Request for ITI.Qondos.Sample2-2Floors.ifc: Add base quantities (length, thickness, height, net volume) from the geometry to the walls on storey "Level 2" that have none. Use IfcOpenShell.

First a look at what the model holds.

```python
import ifcopenshell
import ifcopenshell.util.element
import ifcopenshell.util.unit

model = ifcopenshell.open("ITI.Qondos.Sample2-2Floors.ifc")
print(model.schema)
for unit_type in ("LENGTHUNIT", "AREAUNIT", "VOLUMEUNIT"):
    print(unit_type, ifcopenshell.util.unit.calculate_unit_scale(model, unit_type))
storey = next(s for s in model.by_type("IfcBuildingStorey") if s.Name == "Level 2")
walls = [e for e in ifcopenshell.util.element.get_decomposition(storey) if e.is_a("IfcWall")]
for e in sorted(walls, key=lambda e: e.id()):
    print(e.id(), e.is_a(), e.Name, list(ifcopenshell.util.element.get_psets(e, qtos_only=True)), sep=" | ")
```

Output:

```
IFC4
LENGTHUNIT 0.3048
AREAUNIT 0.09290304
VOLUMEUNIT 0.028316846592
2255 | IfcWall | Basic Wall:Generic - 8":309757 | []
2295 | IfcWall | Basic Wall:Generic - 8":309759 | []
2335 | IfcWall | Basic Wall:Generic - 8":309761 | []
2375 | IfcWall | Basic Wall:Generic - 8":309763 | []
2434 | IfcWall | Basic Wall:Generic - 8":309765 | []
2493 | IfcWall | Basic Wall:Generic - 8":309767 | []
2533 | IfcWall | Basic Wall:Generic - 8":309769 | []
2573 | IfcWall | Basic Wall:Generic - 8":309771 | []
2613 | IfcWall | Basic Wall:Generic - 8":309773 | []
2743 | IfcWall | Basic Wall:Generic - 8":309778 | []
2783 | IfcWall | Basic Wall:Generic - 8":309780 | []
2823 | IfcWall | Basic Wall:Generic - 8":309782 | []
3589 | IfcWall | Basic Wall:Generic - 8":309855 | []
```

```python
import ifcopenshell
import ifcopenshell.api.pset
import ifcopenshell.geom
import ifcopenshell.util.element
import ifcopenshell.util.shape
import ifcopenshell.util.unit

model = ifcopenshell.open("ITI.Qondos.Sample2-2Floors.ifc")
unit_scale = ifcopenshell.util.unit.calculate_unit_scale(model)
volume_scale = ifcopenshell.util.unit.calculate_unit_scale(model, "VOLUMEUNIT")
settings = ifcopenshell.geom.settings()

storey = next(s for s in model.by_type("IfcBuildingStorey") if s.Name == "Level 2")
walls = [e for e in ifcopenshell.util.element.get_decomposition(storey) if e.is_a("IfcWall")]

for e in sorted(walls, key=lambda e: e.id()):
    if ifcopenshell.util.element.get_psets(e, qtos_only=True, should_inherit=False):
        continue
    # Geometry comes back in metres, in the element's own axes.
    shape = ifcopenshell.geom.create_shape(settings, e)
    values = {
        "Length": ifcopenshell.util.shape.get_x(shape.geometry) / unit_scale,
        "Width": ifcopenshell.util.shape.get_y(shape.geometry) / unit_scale,
        "Height": ifcopenshell.util.shape.get_z(shape.geometry) / unit_scale,
        "NetVolume": ifcopenshell.util.shape.get_volume(shape.geometry) / volume_scale,
    }
    qto = ifcopenshell.api.pset.add_qto(model, product=e, name="Qto_WallBaseQuantities")
    ifcopenshell.api.pset.edit_qto(model, qto=qto, properties=values)
    print(e.id(), {k: round(v, 3) for k, v in values.items()})

model.write("ITI.Qondos.Sample2-2Floors-out.ifc")
```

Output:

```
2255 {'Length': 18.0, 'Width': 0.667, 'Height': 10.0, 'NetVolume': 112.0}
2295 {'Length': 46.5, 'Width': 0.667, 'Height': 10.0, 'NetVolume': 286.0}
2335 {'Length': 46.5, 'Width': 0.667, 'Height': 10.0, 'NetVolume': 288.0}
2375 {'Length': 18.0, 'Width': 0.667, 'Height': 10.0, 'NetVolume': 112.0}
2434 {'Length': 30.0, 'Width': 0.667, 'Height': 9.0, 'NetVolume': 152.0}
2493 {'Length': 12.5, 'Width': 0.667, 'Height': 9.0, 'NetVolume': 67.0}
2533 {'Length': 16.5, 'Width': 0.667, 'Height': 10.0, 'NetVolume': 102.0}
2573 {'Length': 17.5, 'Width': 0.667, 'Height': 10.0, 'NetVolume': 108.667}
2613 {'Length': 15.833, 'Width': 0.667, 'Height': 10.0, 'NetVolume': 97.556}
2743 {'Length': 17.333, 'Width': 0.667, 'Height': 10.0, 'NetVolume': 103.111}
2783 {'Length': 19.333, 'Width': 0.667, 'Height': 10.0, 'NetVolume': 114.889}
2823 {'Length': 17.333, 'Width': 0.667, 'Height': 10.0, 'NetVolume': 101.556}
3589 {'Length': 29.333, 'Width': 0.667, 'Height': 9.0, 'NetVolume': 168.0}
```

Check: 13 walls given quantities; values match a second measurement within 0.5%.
